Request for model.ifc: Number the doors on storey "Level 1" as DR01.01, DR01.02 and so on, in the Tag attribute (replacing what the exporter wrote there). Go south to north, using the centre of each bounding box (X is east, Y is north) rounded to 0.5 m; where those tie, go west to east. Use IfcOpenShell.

First a look at what the model holds.

```python
import ifcopenshell
import ifcopenshell.util.element
import ifcopenshell.util.placement

model = ifcopenshell.open("model.ifc")
print(model.schema)
storey = next(s for s in model.by_type("IfcBuildingStorey") if s.Name == "Level 1")
doors = [e for e in ifcopenshell.util.element.get_decomposition(storey) if e.is_a("IfcDoor")]
for e in sorted(doors, key=lambda e: e.id()):
    origin = ifcopenshell.util.placement.get_local_placement(e.ObjectPlacement)[:3, 3]
    print(e.id(), e.Tag, e.Name, origin.round(2) + 0.0, sep=" | ")
```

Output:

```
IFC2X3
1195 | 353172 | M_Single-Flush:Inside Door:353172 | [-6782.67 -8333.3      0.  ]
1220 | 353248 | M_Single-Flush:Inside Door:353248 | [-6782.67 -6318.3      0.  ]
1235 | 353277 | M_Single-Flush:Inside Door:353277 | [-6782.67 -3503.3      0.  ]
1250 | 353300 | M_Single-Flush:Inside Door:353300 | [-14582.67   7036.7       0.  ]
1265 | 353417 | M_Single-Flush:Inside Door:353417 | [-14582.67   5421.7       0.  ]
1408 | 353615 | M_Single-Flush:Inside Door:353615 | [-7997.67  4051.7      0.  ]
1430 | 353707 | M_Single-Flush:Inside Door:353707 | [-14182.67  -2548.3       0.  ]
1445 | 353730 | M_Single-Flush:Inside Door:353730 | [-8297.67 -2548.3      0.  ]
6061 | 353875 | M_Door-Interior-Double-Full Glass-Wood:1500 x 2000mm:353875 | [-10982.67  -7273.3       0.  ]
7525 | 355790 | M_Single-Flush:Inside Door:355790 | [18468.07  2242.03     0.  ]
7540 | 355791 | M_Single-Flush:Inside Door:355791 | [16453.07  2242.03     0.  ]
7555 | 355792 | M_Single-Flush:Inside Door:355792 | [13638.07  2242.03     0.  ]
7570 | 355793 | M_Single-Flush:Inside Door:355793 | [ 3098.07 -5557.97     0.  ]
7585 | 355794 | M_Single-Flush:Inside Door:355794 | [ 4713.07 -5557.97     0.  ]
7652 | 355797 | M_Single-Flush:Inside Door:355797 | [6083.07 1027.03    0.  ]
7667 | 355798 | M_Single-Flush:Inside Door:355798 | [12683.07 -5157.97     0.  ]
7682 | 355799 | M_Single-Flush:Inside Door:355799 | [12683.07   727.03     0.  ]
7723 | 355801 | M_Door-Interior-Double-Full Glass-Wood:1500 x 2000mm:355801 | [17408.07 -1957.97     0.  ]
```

```python
import ifcopenshell
import ifcopenshell.geom
import ifcopenshell.util.element
import ifcopenshell.util.shape

model = ifcopenshell.open("model.ifc")
settings = ifcopenshell.geom.settings()
settings.set("use-world-coords", True)


def centre(element):
    shape = ifcopenshell.geom.create_shape(settings, element)
    return ifcopenshell.util.shape.get_bbox_centroid(shape.geometry)


storey = next(s for s in model.by_type("IfcBuildingStorey") if s.Name == "Level 1")
doors = [e for e in ifcopenshell.util.element.get_decomposition(storey) if e.is_a("IfcDoor")]

# Insertion points can sit at a corner or the storey origin, so sort by the geometry (in metres).
centres = {e: centre(e) for e in doors}
doors.sort(key=lambda e: (round(centres[e][1] / 0.5), centres[e][0]))

for i, e in enumerate(doors, start=1):
    number = f"DR01.{i:02d}"
    e.Tag = number
    print(e.id(), number)

model.write("model_v2.ifc")
```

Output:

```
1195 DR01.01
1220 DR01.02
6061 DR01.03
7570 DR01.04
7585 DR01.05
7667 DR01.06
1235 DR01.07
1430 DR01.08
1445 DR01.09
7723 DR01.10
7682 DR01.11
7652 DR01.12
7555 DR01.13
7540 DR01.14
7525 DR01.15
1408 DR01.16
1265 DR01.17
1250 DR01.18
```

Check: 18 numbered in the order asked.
